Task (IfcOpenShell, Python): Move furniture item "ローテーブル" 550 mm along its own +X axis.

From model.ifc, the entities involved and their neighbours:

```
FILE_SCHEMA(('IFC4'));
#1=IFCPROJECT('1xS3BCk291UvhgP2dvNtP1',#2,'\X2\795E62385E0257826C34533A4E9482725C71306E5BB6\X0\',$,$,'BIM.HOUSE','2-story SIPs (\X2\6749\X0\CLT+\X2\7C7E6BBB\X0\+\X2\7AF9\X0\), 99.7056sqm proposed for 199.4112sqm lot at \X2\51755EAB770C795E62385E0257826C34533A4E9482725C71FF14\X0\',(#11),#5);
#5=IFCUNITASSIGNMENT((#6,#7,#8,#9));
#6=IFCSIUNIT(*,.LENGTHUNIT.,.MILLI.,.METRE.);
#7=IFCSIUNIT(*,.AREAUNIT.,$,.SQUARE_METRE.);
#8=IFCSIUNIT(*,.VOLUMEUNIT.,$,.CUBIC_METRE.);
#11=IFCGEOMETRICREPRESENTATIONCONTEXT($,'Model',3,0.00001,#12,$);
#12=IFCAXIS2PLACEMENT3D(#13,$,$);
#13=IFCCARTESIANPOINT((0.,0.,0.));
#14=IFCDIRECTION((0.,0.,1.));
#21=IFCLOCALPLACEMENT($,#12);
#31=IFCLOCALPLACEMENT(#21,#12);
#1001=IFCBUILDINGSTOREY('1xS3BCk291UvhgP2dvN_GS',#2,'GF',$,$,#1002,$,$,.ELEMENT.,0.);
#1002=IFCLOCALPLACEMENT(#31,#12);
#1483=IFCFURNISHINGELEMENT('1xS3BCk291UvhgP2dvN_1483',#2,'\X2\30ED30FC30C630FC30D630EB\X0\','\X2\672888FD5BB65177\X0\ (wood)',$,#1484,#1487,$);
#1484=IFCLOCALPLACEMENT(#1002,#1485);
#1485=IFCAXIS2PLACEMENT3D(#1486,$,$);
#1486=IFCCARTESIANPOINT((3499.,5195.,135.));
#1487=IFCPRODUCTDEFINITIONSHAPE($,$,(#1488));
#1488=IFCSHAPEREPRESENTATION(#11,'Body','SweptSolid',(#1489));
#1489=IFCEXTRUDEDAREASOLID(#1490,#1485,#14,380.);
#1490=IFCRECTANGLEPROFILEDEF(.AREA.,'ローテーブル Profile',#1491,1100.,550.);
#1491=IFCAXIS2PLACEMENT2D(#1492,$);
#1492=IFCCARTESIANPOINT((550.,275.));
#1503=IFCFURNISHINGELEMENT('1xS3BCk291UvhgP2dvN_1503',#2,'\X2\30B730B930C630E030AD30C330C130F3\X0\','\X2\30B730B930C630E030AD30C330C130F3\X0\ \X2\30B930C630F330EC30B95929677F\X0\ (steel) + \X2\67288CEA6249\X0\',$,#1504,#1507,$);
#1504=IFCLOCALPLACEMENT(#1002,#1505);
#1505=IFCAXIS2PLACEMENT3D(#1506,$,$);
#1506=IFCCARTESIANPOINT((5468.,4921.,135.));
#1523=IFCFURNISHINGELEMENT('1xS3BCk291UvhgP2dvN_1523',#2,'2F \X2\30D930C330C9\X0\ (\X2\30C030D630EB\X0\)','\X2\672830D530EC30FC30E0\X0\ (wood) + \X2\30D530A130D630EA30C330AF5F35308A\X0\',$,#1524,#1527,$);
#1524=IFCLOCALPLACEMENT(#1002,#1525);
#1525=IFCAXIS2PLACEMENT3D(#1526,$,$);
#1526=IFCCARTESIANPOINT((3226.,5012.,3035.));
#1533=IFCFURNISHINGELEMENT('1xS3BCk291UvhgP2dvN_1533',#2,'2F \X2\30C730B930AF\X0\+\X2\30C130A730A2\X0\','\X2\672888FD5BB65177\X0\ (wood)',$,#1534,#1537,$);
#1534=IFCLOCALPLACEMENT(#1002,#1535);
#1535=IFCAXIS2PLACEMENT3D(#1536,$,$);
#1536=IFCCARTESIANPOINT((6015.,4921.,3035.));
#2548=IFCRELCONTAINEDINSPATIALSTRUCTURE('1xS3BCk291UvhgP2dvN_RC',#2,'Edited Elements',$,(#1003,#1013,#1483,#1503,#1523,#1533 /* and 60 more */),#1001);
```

```python
import ifcopenshell
import ifcopenshell.api.geometry
import ifcopenshell.util.placement
import ifcopenshell.util.unit

model = ifcopenshell.open("model.ifc")
unit_scale = ifcopenshell.util.unit.calculate_unit_scale(model)

item = model.by_guid("1xS3BCk291UvhgP2dvN_1483")
matrix = ifcopenshell.util.placement.get_local_placement(item.ObjectPlacement)
matrix[:3, 3] += matrix[:3, 0] * 0.55 / unit_scale
ifcopenshell.api.geometry.edit_object_placement(model, product=item, matrix=matrix, is_si=False)

print(ifcopenshell.util.placement.get_local_placement(item.ObjectPlacement).round(3) + 0.0)

model.write("model_rev.ifc")
```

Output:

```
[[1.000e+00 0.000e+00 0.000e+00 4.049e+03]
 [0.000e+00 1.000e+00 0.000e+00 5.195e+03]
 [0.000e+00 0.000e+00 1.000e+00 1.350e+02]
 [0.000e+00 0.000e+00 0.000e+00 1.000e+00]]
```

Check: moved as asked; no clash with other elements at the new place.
